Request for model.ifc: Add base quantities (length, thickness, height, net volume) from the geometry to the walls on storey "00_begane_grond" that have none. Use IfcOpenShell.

First a look at what the model holds.

```python
import ifcopenshell
import ifcopenshell.util.element
import ifcopenshell.util.unit

model = ifcopenshell.open("model.ifc")
print(model.schema)
for unit_type in ("LENGTHUNIT", "AREAUNIT", "VOLUMEUNIT"):
    print(unit_type, ifcopenshell.util.unit.calculate_unit_scale(model, unit_type))
storey = next(s for s in model.by_type("IfcBuildingStorey") if s.Name == "00_begane_grond")
walls = [e for e in ifcopenshell.util.element.get_decomposition(storey) if e.is_a("IfcWall")]
for e in sorted(walls, key=lambda e: e.id()):
    print(e.id(), e.is_a(), e.Name, list(ifcopenshell.util.element.get_psets(e, qtos_only=True)), sep=" | ")
```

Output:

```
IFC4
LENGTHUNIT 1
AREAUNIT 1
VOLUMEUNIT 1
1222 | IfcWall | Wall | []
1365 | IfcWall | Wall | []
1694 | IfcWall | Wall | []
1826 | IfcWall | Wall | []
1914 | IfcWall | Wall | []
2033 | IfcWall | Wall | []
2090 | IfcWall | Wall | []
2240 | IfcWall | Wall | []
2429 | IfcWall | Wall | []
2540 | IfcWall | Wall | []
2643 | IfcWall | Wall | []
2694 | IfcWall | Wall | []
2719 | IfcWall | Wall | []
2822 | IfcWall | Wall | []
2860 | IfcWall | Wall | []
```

```python
import ifcopenshell
import ifcopenshell.api.pset
import ifcopenshell.geom
import ifcopenshell.util.element
import ifcopenshell.util.shape
import ifcopenshell.util.unit

model = ifcopenshell.open("model.ifc")
unit_scale = ifcopenshell.util.unit.calculate_unit_scale(model)
volume_scale = ifcopenshell.util.unit.calculate_unit_scale(model, "VOLUMEUNIT")
settings = ifcopenshell.geom.settings()

storey = next(s for s in model.by_type("IfcBuildingStorey") if s.Name == "00_begane_grond")
walls = [e for e in ifcopenshell.util.element.get_decomposition(storey) if e.is_a("IfcWall")]

for e in sorted(walls, key=lambda e: e.id()):
    if ifcopenshell.util.element.get_psets(e, qtos_only=True, should_inherit=False):
        continue
    # Geometry comes back in metres, in the element's own axes.
    shape = ifcopenshell.geom.create_shape(settings, e)
    values = {
        "Length": ifcopenshell.util.shape.get_x(shape.geometry) / unit_scale,
        "Width": ifcopenshell.util.shape.get_y(shape.geometry) / unit_scale,
        "Height": ifcopenshell.util.shape.get_z(shape.geometry) / unit_scale,
        "NetVolume": ifcopenshell.util.shape.get_volume(shape.geometry) / volume_scale,
    }
    qto = ifcopenshell.api.pset.add_qto(model, product=e, name="Qto_WallBaseQuantities")
    ifcopenshell.api.pset.edit_qto(model, qto=qto, properties=values)
    print(e.id(), {k: round(v, 3) for k, v in values.items()})

model.write("model_updated.ifc")
```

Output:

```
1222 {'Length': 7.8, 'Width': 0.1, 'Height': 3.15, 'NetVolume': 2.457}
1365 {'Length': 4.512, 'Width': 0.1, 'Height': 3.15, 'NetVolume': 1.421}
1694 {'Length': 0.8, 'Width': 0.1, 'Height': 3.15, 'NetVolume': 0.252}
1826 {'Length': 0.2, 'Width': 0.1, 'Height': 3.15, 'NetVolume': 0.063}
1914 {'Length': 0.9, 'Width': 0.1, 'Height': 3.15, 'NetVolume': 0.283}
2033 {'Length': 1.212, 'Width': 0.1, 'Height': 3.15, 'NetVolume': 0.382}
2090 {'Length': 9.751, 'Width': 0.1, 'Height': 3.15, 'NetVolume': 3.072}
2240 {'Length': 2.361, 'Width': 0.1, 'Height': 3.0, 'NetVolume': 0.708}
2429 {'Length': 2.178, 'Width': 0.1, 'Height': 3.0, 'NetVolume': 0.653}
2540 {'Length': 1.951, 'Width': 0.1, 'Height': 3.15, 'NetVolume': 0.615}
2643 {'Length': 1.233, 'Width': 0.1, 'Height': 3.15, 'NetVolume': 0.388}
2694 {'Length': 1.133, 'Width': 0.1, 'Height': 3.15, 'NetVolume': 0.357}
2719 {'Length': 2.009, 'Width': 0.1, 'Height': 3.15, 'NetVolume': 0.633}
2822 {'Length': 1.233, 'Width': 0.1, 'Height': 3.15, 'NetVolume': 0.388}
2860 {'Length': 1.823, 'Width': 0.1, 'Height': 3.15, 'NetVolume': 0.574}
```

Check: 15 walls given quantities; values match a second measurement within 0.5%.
